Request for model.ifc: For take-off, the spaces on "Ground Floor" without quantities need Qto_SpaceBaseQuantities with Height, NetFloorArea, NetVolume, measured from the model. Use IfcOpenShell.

First a look at what the model holds.

```python
import ifcopenshell
import ifcopenshell.util.element
import ifcopenshell.util.unit

model = ifcopenshell.open("model.ifc")
print(model.schema)
for unit_type in ("LENGTHUNIT", "AREAUNIT", "VOLUMEUNIT"):
    print(unit_type, ifcopenshell.util.unit.calculate_unit_scale(model, unit_type))
storey = next(s for s in model.by_type("IfcBuildingStorey") if s.Name == "Ground Floor")
spaces = [e for e in ifcopenshell.util.element.get_decomposition(storey) if e.is_a("IfcSpace")]
for e in sorted(spaces, key=lambda e: e.id()):
    print(e.id(), e.is_a(), e.Name, list(ifcopenshell.util.element.get_psets(e, qtos_only=True)), sep=" | ")
```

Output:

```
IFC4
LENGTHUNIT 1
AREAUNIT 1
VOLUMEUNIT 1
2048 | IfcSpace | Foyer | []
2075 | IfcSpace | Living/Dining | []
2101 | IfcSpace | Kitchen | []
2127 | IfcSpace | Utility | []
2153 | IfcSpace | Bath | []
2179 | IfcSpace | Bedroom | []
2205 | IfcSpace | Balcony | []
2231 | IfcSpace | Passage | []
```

```python
import ifcopenshell
import ifcopenshell.api.pset
import ifcopenshell.geom
import ifcopenshell.util.element
import ifcopenshell.util.shape
import ifcopenshell.util.unit

model = ifcopenshell.open("model.ifc")
unit_scale = ifcopenshell.util.unit.calculate_unit_scale(model)
area_scale = ifcopenshell.util.unit.calculate_unit_scale(model, "AREAUNIT")
volume_scale = ifcopenshell.util.unit.calculate_unit_scale(model, "VOLUMEUNIT")
settings = ifcopenshell.geom.settings()

storey = next(s for s in model.by_type("IfcBuildingStorey") if s.Name == "Ground Floor")
spaces = [e for e in ifcopenshell.util.element.get_decomposition(storey) if e.is_a("IfcSpace")]

for e in sorted(spaces, key=lambda e: e.id()):
    if ifcopenshell.util.element.get_psets(e, qtos_only=True, should_inherit=False):
        continue
    # Geometry comes back in metres, in the element's own axes.
    shape = ifcopenshell.geom.create_shape(settings, e)
    values = {
        "Height": ifcopenshell.util.shape.get_z(shape.geometry) / unit_scale,
        "NetFloorArea": ifcopenshell.util.shape.get_footprint_area(shape.geometry) / area_scale,
        "NetVolume": ifcopenshell.util.shape.get_volume(shape.geometry) / volume_scale,
    }
    qto = ifcopenshell.api.pset.add_qto(model, product=e, name="Qto_SpaceBaseQuantities")
    ifcopenshell.api.pset.edit_qto(model, qto=qto, properties=values)
    print(e.id(), {k: round(v, 3) for k, v in values.items()})

model.write("model-out.ifc")
```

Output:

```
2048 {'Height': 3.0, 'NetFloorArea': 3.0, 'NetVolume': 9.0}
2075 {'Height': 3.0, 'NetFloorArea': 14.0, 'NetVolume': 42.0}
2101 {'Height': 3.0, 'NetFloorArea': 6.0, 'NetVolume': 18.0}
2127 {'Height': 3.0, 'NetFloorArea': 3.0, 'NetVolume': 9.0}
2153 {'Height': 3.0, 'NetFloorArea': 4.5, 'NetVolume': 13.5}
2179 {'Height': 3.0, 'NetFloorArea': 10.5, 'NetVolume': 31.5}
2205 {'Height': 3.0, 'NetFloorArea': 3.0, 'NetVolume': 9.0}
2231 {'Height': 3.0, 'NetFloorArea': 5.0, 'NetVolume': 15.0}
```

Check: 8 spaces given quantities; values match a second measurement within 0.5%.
